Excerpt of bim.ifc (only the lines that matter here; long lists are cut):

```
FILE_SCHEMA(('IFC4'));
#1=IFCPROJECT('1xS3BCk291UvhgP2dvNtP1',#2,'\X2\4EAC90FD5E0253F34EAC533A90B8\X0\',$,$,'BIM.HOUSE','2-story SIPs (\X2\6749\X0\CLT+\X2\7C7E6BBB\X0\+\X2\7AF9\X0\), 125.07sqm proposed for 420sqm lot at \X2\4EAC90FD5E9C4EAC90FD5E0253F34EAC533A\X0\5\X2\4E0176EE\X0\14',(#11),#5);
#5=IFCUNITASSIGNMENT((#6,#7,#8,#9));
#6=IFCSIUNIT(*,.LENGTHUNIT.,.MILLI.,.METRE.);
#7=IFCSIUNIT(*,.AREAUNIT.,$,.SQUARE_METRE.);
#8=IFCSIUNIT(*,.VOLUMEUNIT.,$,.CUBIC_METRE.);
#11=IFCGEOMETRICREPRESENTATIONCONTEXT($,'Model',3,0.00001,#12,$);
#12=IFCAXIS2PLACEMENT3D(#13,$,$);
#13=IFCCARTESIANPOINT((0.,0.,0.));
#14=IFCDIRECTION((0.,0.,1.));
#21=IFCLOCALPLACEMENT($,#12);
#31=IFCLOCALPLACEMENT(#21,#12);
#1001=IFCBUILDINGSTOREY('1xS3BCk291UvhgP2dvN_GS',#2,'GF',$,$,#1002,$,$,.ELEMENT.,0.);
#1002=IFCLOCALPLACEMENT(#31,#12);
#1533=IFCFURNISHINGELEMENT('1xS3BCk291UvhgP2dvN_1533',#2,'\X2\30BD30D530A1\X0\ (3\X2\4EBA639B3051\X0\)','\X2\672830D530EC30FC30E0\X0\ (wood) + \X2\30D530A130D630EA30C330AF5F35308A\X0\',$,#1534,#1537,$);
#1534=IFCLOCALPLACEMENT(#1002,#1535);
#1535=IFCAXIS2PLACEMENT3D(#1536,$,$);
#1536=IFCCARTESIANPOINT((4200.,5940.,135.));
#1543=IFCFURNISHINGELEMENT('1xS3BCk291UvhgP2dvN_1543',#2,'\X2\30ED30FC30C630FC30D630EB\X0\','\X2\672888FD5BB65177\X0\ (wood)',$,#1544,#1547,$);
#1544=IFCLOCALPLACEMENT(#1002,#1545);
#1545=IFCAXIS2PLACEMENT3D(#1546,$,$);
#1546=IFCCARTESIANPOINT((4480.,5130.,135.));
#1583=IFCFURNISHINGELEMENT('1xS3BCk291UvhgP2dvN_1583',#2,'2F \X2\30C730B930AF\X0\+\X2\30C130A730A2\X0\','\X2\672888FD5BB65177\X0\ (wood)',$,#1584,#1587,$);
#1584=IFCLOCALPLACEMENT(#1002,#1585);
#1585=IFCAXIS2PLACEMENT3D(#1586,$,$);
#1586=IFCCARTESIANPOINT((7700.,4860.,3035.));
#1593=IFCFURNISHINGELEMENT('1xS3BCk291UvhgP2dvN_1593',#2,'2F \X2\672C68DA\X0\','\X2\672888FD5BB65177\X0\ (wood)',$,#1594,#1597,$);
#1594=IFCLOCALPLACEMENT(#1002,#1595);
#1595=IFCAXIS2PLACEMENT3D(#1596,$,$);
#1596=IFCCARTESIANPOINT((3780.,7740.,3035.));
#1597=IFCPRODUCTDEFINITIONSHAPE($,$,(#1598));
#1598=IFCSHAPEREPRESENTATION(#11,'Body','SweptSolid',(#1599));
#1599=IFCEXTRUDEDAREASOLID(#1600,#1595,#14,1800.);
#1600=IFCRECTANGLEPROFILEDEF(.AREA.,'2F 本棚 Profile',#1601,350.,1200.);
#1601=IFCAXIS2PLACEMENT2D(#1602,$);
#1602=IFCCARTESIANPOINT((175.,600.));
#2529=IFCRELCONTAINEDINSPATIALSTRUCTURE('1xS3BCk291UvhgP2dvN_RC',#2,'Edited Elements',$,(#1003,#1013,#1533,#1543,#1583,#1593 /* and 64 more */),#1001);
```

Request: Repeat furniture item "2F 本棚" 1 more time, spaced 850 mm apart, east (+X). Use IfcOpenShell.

```python
import numpy as np
import ifcopenshell
import ifcopenshell.api.geometry
import ifcopenshell.api.root
import ifcopenshell.util.element
import ifcopenshell.util.placement
import ifcopenshell.util.unit

model = ifcopenshell.open("bim.ifc")
unit_scale = ifcopenshell.util.unit.calculate_unit_scale(model)


def reuse_history(source, copy):
    """copy_class also copies each property set's owner history, people and application; keep the originals."""
    for rel in copy.IsDefinedBy:
        if rel.is_a("IfcRelDefinesByProperties") and (history := rel.RelatingPropertyDefinition.OwnerHistory):
            rel.RelatingPropertyDefinition.OwnerHistory = source.OwnerHistory
            ifcopenshell.util.element.remove_deep2(model, history)


source = model.by_guid("1xS3BCk291UvhgP2dvN_1593")
base = ifcopenshell.util.placement.get_local_placement(source.ObjectPlacement)
step = np.array([1.0, 0.0, 0.0]) * 0.85 / unit_scale

for i in range(1, 2):
    copy = ifcopenshell.api.root.copy_class(model, product=source)
    copy.Representation = ifcopenshell.util.element.copy_deep(
        model, source.Representation, exclude=["IfcGeometricRepresentationContext", "IfcRepresentationMap"]
    )
    reuse_history(source, copy)
    matrix = base.copy()
    matrix[:3, 3] += i * step
    print("added at", matrix[:3, 3].round(3) + 0.0)
    ifcopenshell.api.geometry.edit_object_placement(model, product=copy, matrix=matrix, is_si=False)

model.write("bim_updated.ifc")
```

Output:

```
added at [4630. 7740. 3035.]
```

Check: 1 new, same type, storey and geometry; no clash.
